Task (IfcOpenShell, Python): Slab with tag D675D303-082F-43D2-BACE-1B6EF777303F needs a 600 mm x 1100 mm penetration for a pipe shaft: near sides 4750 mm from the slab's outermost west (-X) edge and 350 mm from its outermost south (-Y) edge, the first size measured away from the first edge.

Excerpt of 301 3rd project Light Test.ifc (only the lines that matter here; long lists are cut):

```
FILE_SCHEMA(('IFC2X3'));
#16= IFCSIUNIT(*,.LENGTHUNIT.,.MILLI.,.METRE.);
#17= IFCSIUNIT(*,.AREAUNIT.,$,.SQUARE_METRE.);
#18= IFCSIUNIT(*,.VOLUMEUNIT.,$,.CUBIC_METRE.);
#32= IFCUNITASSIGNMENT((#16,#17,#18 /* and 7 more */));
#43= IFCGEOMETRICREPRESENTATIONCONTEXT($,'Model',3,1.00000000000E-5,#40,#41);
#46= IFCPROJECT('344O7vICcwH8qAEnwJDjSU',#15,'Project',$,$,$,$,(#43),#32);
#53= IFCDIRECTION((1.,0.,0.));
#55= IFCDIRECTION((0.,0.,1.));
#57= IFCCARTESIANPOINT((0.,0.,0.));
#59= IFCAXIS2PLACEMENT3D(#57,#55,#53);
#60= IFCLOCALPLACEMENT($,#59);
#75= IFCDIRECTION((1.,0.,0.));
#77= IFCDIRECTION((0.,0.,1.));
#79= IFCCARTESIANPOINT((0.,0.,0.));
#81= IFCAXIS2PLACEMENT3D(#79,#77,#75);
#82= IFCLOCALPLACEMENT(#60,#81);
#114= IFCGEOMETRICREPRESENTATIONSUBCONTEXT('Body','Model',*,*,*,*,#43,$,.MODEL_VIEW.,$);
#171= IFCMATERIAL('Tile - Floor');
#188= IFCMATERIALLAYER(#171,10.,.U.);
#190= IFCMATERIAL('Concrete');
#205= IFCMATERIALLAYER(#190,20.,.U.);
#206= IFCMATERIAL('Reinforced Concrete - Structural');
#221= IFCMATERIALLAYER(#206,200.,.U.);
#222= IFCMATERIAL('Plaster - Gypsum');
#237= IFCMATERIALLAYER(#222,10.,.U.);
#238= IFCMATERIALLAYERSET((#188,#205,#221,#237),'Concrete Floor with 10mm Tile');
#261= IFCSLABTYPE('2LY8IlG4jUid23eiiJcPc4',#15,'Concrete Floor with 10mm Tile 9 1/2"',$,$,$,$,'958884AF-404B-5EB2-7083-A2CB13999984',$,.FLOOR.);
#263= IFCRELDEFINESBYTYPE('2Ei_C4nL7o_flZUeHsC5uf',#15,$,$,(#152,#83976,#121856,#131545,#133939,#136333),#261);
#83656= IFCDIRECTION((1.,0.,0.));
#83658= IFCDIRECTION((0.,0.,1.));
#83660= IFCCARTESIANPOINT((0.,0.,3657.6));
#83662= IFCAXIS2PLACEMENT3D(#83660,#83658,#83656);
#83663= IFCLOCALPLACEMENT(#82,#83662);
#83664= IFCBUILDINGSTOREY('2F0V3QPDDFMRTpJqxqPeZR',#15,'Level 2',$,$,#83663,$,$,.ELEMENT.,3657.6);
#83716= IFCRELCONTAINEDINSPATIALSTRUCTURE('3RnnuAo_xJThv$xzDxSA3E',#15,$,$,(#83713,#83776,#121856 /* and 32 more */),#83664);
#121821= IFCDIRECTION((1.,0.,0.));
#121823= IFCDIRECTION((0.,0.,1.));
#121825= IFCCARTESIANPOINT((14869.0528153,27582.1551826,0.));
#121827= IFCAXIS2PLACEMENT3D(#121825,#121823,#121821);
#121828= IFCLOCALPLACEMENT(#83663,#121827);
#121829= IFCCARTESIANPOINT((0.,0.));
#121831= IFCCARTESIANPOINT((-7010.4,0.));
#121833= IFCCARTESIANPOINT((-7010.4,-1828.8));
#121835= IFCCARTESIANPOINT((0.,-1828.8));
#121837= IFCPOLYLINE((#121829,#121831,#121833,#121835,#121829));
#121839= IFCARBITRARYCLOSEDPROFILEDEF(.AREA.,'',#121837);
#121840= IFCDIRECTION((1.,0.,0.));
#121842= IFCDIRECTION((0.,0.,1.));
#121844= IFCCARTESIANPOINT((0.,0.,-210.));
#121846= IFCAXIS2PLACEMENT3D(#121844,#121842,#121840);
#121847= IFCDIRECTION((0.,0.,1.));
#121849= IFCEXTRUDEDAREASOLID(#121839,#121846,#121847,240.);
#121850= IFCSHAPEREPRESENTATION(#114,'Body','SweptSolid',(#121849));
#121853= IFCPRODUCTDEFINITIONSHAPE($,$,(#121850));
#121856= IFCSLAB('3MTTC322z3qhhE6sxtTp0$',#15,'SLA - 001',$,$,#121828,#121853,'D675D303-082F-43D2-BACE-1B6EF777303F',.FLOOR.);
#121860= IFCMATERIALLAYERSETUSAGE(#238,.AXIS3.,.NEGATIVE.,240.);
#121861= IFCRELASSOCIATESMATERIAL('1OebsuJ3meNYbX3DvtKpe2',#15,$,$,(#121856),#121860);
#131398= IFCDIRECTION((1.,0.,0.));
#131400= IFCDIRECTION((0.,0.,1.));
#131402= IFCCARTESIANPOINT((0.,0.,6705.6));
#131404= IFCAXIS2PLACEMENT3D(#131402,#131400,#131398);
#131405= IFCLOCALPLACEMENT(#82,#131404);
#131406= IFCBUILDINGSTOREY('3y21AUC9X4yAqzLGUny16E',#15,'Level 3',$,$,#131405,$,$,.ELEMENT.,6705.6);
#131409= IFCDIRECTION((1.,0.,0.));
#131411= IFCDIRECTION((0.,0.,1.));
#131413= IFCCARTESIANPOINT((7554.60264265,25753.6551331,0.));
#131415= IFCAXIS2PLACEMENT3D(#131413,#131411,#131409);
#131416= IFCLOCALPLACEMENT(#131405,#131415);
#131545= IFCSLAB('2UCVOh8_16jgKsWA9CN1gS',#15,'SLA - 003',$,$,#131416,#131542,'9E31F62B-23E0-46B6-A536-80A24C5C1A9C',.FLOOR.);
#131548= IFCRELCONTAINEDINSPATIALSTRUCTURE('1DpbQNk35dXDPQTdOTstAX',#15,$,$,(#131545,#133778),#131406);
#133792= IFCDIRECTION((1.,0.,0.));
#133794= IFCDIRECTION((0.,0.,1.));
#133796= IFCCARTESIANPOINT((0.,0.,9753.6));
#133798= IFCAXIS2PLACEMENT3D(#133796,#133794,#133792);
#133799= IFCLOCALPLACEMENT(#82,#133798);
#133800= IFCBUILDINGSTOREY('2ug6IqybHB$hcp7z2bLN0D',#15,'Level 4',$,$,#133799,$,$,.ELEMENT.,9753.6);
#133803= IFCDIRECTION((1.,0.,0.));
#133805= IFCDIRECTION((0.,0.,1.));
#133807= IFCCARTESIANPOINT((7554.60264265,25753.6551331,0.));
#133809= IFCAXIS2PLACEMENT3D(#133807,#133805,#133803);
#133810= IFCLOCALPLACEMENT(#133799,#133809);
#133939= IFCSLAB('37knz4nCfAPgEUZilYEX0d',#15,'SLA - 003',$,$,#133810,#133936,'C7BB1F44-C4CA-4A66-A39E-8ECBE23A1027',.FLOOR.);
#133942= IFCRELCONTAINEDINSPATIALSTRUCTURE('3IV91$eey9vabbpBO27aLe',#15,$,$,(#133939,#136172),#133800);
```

```python
import numpy as np
import ifcopenshell
import ifcopenshell.api.feature
import ifcopenshell.api.geometry
import ifcopenshell.api.root
import ifcopenshell.geom
import ifcopenshell.util.placement
import ifcopenshell.util.representation
import ifcopenshell.util.shape
import ifcopenshell.util.unit

model = ifcopenshell.open("301 3rd project Light Test.ifc")
unit_scale = ifcopenshell.util.unit.calculate_unit_scale(model)
settings = ifcopenshell.geom.settings()


def volume(element):
    """Net volume in cubic metres, openings subtracted."""
    shape = ifcopenshell.geom.create_shape(settings, element)
    return ifcopenshell.util.shape.get_volume(shape.geometry)


slab = model.by_guid("3MTTC322z3qhhE6sxtTp0$")
before = volume(slab)

# Extent in the slab's own axes, in metres. The edges named are its -X and -Y sides.
slab_shape = ifcopenshell.geom.create_shape(settings, slab)
vertices = ifcopenshell.util.shape.get_vertices(slab_shape.geometry)
x_min, y_min, bottom = vertices.min(axis=0)
top = vertices[:, 2].max()

opening = ifcopenshell.api.root.create_entity(model, ifc_class="IfcOpeningElement", name="Pipe shaft opening")
context = ifcopenshell.util.representation.get_context(model, "Model", "Body", "MODEL_VIEW")
width, depth = 0.6, 1.1
outline = [(0.0, 0.0), (width, 0.0), (width, depth), (0.0, depth), (0.0, 0.0)]
# Overshoot both faces by 50 mm so the cut is clean.
shape = ifcopenshell.api.geometry.add_slab_representation(
    model, context=context, depth=top - bottom + 0.1, polyline=outline
)
ifcopenshell.api.geometry.assign_representation(model, product=opening, representation=shape)

matrix = ifcopenshell.util.placement.get_local_placement(slab.ObjectPlacement)
matrix[:, 3] = matrix @ np.append(np.array([x_min + 4.75, y_min + 0.35, bottom - 0.05]) / unit_scale, 1.0)
ifcopenshell.api.geometry.edit_object_placement(model, product=opening, matrix=matrix, is_si=False)
ifcopenshell.api.feature.add_feature(model, feature=opening, element=slab)

after = volume(slab)

print(f"slab volume {before:.3f} -> {after:.3f} m3")

model.write("301 3rd project Light Test-out.ifc")
```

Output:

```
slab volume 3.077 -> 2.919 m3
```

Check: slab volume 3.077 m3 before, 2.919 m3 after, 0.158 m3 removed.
